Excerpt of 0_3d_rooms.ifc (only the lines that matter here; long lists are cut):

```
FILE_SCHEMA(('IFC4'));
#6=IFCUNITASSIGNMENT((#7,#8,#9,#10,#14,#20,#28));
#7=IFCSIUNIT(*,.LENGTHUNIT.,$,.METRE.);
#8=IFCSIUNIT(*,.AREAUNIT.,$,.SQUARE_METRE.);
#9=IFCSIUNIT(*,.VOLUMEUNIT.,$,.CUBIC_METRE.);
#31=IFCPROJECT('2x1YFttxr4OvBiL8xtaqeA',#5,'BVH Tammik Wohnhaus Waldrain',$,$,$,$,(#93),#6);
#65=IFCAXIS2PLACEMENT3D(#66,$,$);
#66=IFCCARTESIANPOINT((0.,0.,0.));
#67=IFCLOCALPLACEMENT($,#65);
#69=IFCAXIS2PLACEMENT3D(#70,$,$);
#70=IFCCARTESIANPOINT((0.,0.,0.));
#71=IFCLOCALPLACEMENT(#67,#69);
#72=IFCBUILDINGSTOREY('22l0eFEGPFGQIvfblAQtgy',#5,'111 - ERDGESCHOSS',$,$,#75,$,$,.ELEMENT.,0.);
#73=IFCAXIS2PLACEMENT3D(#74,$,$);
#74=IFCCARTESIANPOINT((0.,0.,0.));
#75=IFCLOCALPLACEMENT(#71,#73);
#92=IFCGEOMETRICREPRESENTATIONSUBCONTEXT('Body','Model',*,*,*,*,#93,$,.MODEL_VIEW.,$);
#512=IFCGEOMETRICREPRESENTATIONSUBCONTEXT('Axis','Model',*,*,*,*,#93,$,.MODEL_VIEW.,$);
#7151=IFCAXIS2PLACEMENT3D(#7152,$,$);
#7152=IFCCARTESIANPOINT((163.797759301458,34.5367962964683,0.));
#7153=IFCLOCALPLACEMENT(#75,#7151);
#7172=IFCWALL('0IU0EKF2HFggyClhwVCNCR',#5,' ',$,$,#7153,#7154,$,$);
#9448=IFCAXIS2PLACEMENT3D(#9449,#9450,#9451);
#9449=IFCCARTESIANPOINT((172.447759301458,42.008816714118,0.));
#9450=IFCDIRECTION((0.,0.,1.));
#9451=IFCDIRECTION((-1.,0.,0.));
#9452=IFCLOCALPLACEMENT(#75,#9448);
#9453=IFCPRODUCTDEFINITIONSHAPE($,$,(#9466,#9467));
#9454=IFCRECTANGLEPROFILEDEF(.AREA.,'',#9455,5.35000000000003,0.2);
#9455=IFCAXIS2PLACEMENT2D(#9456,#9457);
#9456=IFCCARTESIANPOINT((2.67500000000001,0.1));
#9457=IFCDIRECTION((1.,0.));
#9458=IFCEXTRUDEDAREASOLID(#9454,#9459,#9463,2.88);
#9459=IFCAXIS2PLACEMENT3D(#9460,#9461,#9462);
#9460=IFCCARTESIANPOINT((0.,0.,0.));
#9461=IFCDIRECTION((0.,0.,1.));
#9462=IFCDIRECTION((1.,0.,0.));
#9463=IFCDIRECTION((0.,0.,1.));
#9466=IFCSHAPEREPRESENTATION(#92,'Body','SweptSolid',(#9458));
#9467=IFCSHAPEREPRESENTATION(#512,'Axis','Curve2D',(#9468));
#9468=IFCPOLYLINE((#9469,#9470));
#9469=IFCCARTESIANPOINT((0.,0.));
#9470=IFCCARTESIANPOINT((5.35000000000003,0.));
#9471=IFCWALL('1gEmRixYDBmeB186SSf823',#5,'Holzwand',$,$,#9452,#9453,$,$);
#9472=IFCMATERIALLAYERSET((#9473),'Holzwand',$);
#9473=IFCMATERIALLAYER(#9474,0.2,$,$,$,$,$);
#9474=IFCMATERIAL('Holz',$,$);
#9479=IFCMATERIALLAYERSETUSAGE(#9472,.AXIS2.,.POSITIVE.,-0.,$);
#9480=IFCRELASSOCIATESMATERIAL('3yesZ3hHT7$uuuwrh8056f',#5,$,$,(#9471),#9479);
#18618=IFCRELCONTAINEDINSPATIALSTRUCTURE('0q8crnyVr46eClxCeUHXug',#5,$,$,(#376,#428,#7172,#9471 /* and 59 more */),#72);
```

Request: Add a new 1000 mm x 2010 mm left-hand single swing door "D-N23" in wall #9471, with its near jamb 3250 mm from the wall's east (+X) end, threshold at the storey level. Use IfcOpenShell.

```python
import numpy as np
import ifcopenshell
import ifcopenshell.api.feature
import ifcopenshell.api.geometry
import ifcopenshell.api.root
import ifcopenshell.api.spatial
import ifcopenshell.geom
import ifcopenshell.util.element
import ifcopenshell.util.placement
import ifcopenshell.util.representation
import ifcopenshell.util.shape
import ifcopenshell.util.unit

model = ifcopenshell.open("0_3d_rooms.ifc")
unit_scale = ifcopenshell.util.unit.calculate_unit_scale(model)
settings = ifcopenshell.geom.settings()


def volume(element):
    """Net volume in cubic metres, openings subtracted."""
    shape = ifcopenshell.geom.create_shape(settings, element)
    return ifcopenshell.util.shape.get_volume(shape.geometry)


wall = model.by_id(9471)
storey = ifcopenshell.util.element.get_container(wall, ifc_class="IfcBuildingStorey")
context = ifcopenshell.util.representation.get_context(model, "Model", "Body", "MODEL_VIEW")
before = volume(wall)

width, height, from_end, sill = 1, 2.01, 3.25, 0.0  # metres

# The wall runs along its own X axis, and the end named is its -X end.
wall_shape = ifcopenshell.geom.create_shape(settings, wall)
x, y, z = ifcopenshell.util.shape.get_vertices(wall_shape.geometry).T
start = x.min() + from_end
face, thickness = float(y.min()), float(y.max() - y.min())
wall_matrix = ifcopenshell.util.placement.get_local_placement(wall.ObjectPlacement)
level = ifcopenshell.util.placement.get_local_placement(storey.ObjectPlacement)[2, 3]


def in_wall(x, y):
    """Placement at x, y metres in the wall's axes, at sill height."""
    matrix = wall_matrix.copy()
    matrix[:, 3] = wall_matrix @ np.array([x / unit_scale, y / unit_scale, 0.0, 1.0])
    matrix[2, 3] = level + sill / unit_scale
    return matrix


# Opening: a box that overshoots both wall faces by 50 mm.
opening = ifcopenshell.api.root.create_entity(model, ifc_class="IfcOpeningElement", predefined_type="OPENING")
box = ifcopenshell.api.geometry.add_wall_representation(
    model, context=context, length=width, height=height, thickness=thickness + 0.1
)
ifcopenshell.api.geometry.assign_representation(model, product=opening, representation=box)
ifcopenshell.api.geometry.edit_object_placement(model, product=opening, matrix=in_wall(start, face - 0.05), is_si=False)
ifcopenshell.api.feature.add_feature(model, feature=opening, element=wall)

door = ifcopenshell.api.root.create_entity(model, ifc_class="IfcDoor", name="D-N23", predefined_type="DOOR")
door.OverallWidth, door.OverallHeight = width / unit_scale, height / unit_scale
door.OperationType = "SINGLE_SWING_LEFT"
body = ifcopenshell.api.geometry.add_door_representation(
    model,
    context=context,
    overall_width=door.OverallWidth,
    overall_height=door.OverallHeight,
    operation_type="SINGLE_SWING_LEFT",
    lining_properties={"LiningDepth": thickness / unit_scale, "ThresholdDepth": thickness / unit_scale},
)
ifcopenshell.api.geometry.assign_representation(model, product=door, representation=body)
ifcopenshell.api.spatial.assign_container(model, products=[door], relating_structure=storey)
ifcopenshell.api.feature.add_filling(model, opening=opening, element=door)

# The lining spans the wall, so the door starts at the wall face.
ifcopenshell.api.geometry.edit_object_placement(model, product=door, matrix=in_wall(start, face), is_si=False)

after = volume(wall)

print(f"wall volume {before:.3f} -> {after:.3f} m3")

model.write("0_3d_rooms_updated.ifc")
```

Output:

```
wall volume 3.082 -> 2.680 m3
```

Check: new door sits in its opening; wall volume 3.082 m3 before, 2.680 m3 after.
